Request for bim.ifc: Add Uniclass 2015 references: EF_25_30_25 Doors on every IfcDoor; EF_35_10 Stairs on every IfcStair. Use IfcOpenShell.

First a look at what the model holds.

```python
import ifcopenshell

model = ifcopenshell.open("bim.ifc")
print(model.schema)
print("classifications:", [c.Name for c in model.by_type("IfcClassification")])
for ifc_class in ("IfcDoor", "IfcRoof", "IfcStair", "IfcWall", "IfcWindow"):
    print(ifc_class, len(model.by_type(ifc_class)))
```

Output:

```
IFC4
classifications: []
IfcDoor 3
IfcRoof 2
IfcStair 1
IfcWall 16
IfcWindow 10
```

```python
import ifcopenshell
import ifcopenshell.api.classification

model = ifcopenshell.open("bim.ifc")

system = ifcopenshell.api.classification.add_classification(model, classification="Uniclass 2015")

codes = {
    "IfcDoor": ("EF_25_30_25", "Doors"),
    "IfcStair": ("EF_35_10", "Stairs"),
}
for ifc_class, (code, name) in codes.items():
    products = model.by_type(ifc_class)
    ifcopenshell.api.classification.add_reference(
        model, products=products, classification=system, identification=code, name=name
    )
    print(code, len(products))

model.write("bim_updated.ifc")
```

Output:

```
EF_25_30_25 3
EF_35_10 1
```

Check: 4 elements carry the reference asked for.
